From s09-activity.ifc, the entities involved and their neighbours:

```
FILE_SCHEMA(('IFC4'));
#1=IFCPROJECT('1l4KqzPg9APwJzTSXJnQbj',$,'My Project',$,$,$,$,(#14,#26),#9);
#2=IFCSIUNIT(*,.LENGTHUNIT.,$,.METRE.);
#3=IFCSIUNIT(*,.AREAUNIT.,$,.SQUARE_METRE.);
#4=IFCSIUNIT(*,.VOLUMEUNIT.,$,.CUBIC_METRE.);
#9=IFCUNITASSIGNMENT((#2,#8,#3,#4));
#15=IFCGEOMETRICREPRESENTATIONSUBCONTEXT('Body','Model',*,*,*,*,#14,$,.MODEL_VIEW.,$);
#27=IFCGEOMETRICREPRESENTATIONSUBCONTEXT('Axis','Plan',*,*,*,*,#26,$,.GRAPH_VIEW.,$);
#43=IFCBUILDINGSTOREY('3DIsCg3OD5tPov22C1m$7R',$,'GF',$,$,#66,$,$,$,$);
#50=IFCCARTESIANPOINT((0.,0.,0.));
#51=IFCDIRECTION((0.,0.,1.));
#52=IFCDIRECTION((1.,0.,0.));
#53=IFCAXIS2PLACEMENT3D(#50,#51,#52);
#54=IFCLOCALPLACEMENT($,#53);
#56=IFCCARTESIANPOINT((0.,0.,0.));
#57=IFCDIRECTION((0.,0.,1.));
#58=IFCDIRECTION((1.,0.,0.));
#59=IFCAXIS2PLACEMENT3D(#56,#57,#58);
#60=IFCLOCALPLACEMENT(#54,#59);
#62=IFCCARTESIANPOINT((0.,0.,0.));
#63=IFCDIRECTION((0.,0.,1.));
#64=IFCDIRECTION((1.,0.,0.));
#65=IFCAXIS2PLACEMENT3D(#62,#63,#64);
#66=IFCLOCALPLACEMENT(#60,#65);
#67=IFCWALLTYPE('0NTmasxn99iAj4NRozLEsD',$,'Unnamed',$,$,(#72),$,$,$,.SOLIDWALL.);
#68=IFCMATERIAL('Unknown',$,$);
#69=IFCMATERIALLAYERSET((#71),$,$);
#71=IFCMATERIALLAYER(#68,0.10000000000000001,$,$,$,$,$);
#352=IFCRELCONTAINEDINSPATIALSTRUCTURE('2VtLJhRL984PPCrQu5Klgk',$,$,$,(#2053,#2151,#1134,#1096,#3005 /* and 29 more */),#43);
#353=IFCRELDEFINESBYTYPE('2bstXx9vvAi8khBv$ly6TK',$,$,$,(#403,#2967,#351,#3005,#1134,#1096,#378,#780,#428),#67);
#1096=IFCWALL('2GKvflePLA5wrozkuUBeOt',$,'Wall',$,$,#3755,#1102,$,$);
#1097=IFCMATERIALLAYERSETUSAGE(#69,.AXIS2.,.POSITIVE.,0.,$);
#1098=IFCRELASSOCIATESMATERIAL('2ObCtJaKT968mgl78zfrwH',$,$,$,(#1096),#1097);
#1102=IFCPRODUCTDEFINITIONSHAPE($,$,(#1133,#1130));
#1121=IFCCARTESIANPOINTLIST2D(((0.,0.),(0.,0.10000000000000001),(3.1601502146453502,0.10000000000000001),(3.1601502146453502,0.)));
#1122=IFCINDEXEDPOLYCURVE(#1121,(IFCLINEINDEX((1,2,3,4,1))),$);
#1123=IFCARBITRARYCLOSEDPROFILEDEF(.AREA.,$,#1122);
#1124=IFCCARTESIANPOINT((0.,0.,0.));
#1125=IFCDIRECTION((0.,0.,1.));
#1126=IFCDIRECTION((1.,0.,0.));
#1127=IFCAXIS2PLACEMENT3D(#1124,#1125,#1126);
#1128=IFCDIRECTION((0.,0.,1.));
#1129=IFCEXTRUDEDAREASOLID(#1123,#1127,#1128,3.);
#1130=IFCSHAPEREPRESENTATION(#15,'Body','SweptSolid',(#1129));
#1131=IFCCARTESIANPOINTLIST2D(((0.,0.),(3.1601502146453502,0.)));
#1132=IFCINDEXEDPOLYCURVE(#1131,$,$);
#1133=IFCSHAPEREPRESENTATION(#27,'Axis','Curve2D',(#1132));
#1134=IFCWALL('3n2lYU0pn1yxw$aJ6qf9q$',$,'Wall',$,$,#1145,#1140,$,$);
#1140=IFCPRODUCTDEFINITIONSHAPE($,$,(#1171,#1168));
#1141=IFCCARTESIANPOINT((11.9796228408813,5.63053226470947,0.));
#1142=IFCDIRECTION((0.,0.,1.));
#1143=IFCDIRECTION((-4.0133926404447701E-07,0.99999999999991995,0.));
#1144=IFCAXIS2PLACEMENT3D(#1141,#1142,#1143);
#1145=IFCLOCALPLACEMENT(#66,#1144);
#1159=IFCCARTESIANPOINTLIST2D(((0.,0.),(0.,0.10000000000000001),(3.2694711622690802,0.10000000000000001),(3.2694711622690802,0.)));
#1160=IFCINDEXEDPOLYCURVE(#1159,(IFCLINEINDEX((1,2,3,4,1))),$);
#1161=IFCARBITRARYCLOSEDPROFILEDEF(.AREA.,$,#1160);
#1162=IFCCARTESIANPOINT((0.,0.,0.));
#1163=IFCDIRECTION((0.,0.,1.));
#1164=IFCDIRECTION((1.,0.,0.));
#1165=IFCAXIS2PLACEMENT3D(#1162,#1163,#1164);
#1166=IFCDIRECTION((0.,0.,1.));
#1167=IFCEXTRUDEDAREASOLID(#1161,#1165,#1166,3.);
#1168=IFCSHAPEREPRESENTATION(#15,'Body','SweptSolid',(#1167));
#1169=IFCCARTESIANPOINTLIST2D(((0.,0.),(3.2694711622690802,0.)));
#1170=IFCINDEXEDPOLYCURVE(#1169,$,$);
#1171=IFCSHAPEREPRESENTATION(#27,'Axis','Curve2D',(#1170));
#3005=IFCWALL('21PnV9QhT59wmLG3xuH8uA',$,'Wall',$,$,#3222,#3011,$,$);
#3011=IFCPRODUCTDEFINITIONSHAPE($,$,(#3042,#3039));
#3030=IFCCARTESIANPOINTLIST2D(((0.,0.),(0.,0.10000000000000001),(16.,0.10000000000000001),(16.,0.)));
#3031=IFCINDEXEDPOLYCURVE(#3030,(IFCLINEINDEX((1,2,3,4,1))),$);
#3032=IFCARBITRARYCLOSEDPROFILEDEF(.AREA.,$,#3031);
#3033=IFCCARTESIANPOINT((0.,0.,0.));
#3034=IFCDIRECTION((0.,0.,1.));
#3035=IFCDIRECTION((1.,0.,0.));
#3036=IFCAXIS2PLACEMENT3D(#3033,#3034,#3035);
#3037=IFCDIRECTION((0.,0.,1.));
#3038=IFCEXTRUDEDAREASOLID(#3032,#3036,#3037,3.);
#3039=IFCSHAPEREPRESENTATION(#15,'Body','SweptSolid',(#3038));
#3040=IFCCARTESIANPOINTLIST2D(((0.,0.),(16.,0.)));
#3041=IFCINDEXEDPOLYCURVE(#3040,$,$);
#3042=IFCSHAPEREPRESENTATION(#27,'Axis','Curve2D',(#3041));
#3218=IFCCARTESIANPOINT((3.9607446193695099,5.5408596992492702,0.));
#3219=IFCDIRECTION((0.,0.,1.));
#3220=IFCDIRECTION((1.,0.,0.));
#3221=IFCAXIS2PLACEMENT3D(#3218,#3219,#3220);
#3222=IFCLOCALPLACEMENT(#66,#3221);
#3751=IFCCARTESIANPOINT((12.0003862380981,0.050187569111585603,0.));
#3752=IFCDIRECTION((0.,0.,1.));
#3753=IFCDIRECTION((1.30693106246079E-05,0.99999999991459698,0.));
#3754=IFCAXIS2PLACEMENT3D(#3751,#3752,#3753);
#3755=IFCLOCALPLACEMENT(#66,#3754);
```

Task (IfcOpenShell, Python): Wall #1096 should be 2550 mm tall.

```python
import ifcopenshell
import ifcopenshell.geom
import ifcopenshell.util.representation
import ifcopenshell.util.shape

model = ifcopenshell.open("s09-activity.ifc")
settings = ifcopenshell.geom.settings()


def volume(element):
    """Net volume in cubic metres, openings subtracted."""
    shape = ifcopenshell.geom.create_shape(settings, element)
    return ifcopenshell.util.shape.get_volume(shape.geometry)


wall = model.by_guid("2GKvflePLA5wrozkuUBeOt")
before = volume(wall)

body = ifcopenshell.util.representation.get_representation(wall, "Model", "Body")
solid = body.Items[0]
old_height = solid.Depth
solid.Depth = 2.55
after = volume(wall)

print(f"height {old_height:g} -> {solid.Depth:g}, volume {before:.3f} -> {after:.3f} m3")

model.write("s09-activity-out.ifc")
```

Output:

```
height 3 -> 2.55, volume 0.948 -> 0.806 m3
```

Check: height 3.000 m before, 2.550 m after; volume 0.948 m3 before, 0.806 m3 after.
